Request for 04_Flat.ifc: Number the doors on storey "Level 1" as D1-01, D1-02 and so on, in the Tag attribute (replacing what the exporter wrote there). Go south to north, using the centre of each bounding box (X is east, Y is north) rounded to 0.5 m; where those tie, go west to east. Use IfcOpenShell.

First a look at what the model holds.

```python
import ifcopenshell
import ifcopenshell.util.element
import ifcopenshell.util.placement

model = ifcopenshell.open("04_Flat.ifc")
print(model.schema)
storey = next(s for s in model.by_type("IfcBuildingStorey") if s.Name == "Level 1")
doors = [e for e in ifcopenshell.util.element.get_decomposition(storey) if e.is_a("IfcDoor")]
for e in sorted(doors, key=lambda e: e.id()):
    origin = ifcopenshell.util.placement.get_local_placement(e.ObjectPlacement)[:3, 3]
    print(e.id(), e.Tag, e.Name, origin.round(2) + 0.0, sep=" | ")
```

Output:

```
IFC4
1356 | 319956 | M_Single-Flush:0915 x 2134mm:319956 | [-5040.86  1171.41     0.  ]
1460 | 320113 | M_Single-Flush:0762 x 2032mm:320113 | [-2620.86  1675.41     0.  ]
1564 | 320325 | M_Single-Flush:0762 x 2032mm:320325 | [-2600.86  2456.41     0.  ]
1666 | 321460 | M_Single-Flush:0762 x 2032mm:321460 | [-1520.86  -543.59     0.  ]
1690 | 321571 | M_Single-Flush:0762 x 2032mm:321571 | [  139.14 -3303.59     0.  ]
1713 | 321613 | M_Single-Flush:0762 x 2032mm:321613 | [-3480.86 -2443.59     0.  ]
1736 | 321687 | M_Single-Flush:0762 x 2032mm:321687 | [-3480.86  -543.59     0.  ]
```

```python
import ifcopenshell
import ifcopenshell.geom
import ifcopenshell.util.element
import ifcopenshell.util.shape

model = ifcopenshell.open("04_Flat.ifc")
settings = ifcopenshell.geom.settings()
settings.set("use-world-coords", True)


def centre(element):
    shape = ifcopenshell.geom.create_shape(settings, element)
    return ifcopenshell.util.shape.get_bbox_centroid(shape.geometry)


storey = next(s for s in model.by_type("IfcBuildingStorey") if s.Name == "Level 1")
doors = [e for e in ifcopenshell.util.element.get_decomposition(storey) if e.is_a("IfcDoor")]

# Insertion points can sit at a corner or the storey origin, so sort by the geometry (in metres).
centres = {e: centre(e) for e in doors}
doors.sort(key=lambda e: (round(centres[e][1] / 0.5), centres[e][0]))

for i, e in enumerate(doors, start=1):
    number = f"D1-{i:02d}"
    e.Tag = number
    print(e.id(), number)

model.write("04_Flat_v2.ifc")
```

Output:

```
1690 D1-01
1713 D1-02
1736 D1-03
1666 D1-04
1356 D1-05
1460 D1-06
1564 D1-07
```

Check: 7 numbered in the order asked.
